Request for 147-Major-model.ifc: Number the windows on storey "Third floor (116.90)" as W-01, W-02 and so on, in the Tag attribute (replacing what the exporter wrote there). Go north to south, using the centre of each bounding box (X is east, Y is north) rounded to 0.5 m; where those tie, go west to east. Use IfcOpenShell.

First a look at what the model holds.

```python
import ifcopenshell
import ifcopenshell.util.element
import ifcopenshell.util.placement

model = ifcopenshell.open("147-Major-model.ifc")
print(model.schema)
storey = next(s for s in model.by_type("IfcBuildingStorey") if s.Name == "Third floor (116.90)")
windows = [e for e in ifcopenshell.util.element.get_decomposition(storey) if e.is_a("IfcWindow")]
for e in sorted(windows, key=lambda e: e.id()):
    origin = ifcopenshell.util.placement.get_local_placement(e.ObjectPlacement)[:3, 3]
    print(e.id(), e.Tag, e.Name, origin.round(2) + 0.0, sep=" | ")
```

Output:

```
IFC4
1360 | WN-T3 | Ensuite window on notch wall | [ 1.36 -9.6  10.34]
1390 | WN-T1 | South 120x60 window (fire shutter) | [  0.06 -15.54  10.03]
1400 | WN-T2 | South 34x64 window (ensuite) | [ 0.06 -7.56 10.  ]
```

```python
import ifcopenshell
import ifcopenshell.geom
import ifcopenshell.util.element
import ifcopenshell.util.shape

model = ifcopenshell.open("147-Major-model.ifc")
settings = ifcopenshell.geom.settings()
settings.set("use-world-coords", True)


def centre(element):
    shape = ifcopenshell.geom.create_shape(settings, element)
    return ifcopenshell.util.shape.get_bbox_centroid(shape.geometry)


storey = next(s for s in model.by_type("IfcBuildingStorey") if s.Name == "Third floor (116.90)")
windows = [e for e in ifcopenshell.util.element.get_decomposition(storey) if e.is_a("IfcWindow")]

# Insertion points can sit at a corner or the storey origin, so sort by the geometry (in metres).
centres = {e: centre(e) for e in windows}
windows.sort(key=lambda e: (-round(centres[e][1] / 0.5), centres[e][0]))

for i, e in enumerate(windows, start=1):
    number = f"W-{i:02d}"
    e.Tag = number
    print(e.id(), number)

model.write("147-Major-model-out.ifc")
```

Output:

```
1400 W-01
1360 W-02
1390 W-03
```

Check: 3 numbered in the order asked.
